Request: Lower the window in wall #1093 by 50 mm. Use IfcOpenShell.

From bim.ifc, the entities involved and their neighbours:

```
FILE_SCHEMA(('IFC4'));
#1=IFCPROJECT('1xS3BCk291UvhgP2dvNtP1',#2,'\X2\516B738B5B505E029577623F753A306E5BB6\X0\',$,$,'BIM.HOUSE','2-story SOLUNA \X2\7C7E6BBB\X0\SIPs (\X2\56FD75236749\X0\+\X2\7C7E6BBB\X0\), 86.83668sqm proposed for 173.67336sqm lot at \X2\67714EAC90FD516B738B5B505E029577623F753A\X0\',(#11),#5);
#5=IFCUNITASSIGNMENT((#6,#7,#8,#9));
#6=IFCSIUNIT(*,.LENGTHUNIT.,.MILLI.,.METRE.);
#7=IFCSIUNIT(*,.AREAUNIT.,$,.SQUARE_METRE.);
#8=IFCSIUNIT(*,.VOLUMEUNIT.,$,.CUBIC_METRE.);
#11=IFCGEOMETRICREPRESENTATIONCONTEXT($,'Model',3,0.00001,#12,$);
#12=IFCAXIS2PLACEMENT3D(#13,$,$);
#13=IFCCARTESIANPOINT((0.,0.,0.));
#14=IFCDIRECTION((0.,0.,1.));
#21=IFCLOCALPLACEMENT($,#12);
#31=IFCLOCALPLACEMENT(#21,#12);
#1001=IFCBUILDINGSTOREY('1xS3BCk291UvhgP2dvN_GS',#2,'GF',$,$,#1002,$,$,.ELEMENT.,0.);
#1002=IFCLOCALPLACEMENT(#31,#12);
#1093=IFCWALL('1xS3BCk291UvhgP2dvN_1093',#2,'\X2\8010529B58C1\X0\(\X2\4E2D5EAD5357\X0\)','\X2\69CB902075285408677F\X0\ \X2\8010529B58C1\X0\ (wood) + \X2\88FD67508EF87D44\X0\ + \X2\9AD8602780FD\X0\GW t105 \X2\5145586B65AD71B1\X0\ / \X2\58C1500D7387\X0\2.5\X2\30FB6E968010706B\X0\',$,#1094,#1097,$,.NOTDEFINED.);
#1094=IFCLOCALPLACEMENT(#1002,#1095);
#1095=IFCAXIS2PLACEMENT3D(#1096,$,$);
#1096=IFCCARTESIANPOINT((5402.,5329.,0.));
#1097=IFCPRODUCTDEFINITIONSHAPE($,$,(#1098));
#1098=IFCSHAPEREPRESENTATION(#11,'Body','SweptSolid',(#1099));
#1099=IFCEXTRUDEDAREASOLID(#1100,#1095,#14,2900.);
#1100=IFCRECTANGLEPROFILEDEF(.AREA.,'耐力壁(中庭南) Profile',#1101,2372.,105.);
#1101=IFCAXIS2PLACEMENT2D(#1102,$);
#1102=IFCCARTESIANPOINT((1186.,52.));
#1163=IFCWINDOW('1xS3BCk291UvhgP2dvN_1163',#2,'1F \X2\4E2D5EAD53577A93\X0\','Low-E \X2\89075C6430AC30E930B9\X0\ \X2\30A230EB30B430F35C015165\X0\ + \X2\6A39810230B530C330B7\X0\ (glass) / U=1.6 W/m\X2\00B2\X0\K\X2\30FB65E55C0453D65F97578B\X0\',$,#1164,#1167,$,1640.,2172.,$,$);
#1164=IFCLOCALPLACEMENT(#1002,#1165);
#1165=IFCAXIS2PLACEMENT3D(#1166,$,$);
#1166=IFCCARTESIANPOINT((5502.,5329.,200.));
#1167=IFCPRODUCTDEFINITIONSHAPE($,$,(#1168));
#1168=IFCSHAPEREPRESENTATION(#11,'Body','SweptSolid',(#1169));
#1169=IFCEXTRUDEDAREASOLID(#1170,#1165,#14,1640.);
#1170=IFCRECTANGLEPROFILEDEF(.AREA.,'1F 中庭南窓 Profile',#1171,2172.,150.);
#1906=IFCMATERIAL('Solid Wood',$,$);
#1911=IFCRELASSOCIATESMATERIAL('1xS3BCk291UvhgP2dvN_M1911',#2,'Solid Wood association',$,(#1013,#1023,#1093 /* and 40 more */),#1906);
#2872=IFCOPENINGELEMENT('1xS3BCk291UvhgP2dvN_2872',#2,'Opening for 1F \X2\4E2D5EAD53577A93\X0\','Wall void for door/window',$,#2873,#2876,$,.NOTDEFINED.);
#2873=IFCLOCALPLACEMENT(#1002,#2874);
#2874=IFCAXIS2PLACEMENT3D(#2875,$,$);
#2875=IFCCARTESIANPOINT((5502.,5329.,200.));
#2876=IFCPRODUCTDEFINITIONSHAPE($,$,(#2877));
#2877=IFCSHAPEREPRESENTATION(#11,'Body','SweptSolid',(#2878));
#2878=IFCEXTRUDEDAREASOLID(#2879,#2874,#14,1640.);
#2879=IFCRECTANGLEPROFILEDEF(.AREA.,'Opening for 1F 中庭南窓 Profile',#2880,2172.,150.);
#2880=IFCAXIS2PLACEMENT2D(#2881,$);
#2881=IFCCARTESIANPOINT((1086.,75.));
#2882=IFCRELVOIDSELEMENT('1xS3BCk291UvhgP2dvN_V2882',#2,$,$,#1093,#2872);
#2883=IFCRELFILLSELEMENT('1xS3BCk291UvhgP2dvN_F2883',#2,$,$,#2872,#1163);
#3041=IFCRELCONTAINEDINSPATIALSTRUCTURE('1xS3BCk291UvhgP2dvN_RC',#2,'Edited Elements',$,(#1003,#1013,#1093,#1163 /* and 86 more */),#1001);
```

```python
import numpy as np
import ifcopenshell
import ifcopenshell.api.geometry
import ifcopenshell.util.placement
import ifcopenshell.util.unit

model = ifcopenshell.open("bim.ifc")
unit_scale = ifcopenshell.util.unit.calculate_unit_scale(model)

window = model.by_id(1163)
opening = window.FillsVoids[0].RelatingOpeningElement
dz = -0.05 / unit_scale

shift = np.array([0.0, 0.0, dz])
# The window is not placed relative to its opening, so move both.
for product in (opening, window):
    matrix = ifcopenshell.util.placement.get_local_placement(product.ObjectPlacement)
    matrix[:3, 3] += shift
    ifcopenshell.api.geometry.edit_object_placement(model, product=product, matrix=matrix, is_si=False)

print(f"moved by {dz * unit_scale:+.3f} m")

model.write("bim_edited.ifc")
```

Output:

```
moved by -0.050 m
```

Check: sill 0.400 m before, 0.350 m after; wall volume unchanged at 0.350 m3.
